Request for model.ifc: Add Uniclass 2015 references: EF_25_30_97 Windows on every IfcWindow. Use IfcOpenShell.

First a look at what the model holds.

```python
import ifcopenshell

model = ifcopenshell.open("model.ifc")
print(model.schema)
print("classifications:", [c.Name for c in model.by_type("IfcClassification")])
for ifc_class in ("IfcDoor", "IfcRoof", "IfcStair", "IfcWall", "IfcWindow"):
    print(ifc_class, len(model.by_type(ifc_class)))
```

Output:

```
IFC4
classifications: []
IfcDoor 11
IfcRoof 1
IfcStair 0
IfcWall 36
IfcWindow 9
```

```python
import ifcopenshell
import ifcopenshell.api.classification

model = ifcopenshell.open("model.ifc")

system = ifcopenshell.api.classification.add_classification(model, classification="Uniclass 2015")

codes = {
    "IfcWindow": ("EF_25_30_97", "Windows"),
}
for ifc_class, (code, name) in codes.items():
    products = model.by_type(ifc_class)
    ifcopenshell.api.classification.add_reference(
        model, products=products, classification=system, identification=code, name=name
    )
    print(code, len(products))

model.write("model_v2.ifc")
```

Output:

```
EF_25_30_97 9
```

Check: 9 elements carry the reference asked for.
